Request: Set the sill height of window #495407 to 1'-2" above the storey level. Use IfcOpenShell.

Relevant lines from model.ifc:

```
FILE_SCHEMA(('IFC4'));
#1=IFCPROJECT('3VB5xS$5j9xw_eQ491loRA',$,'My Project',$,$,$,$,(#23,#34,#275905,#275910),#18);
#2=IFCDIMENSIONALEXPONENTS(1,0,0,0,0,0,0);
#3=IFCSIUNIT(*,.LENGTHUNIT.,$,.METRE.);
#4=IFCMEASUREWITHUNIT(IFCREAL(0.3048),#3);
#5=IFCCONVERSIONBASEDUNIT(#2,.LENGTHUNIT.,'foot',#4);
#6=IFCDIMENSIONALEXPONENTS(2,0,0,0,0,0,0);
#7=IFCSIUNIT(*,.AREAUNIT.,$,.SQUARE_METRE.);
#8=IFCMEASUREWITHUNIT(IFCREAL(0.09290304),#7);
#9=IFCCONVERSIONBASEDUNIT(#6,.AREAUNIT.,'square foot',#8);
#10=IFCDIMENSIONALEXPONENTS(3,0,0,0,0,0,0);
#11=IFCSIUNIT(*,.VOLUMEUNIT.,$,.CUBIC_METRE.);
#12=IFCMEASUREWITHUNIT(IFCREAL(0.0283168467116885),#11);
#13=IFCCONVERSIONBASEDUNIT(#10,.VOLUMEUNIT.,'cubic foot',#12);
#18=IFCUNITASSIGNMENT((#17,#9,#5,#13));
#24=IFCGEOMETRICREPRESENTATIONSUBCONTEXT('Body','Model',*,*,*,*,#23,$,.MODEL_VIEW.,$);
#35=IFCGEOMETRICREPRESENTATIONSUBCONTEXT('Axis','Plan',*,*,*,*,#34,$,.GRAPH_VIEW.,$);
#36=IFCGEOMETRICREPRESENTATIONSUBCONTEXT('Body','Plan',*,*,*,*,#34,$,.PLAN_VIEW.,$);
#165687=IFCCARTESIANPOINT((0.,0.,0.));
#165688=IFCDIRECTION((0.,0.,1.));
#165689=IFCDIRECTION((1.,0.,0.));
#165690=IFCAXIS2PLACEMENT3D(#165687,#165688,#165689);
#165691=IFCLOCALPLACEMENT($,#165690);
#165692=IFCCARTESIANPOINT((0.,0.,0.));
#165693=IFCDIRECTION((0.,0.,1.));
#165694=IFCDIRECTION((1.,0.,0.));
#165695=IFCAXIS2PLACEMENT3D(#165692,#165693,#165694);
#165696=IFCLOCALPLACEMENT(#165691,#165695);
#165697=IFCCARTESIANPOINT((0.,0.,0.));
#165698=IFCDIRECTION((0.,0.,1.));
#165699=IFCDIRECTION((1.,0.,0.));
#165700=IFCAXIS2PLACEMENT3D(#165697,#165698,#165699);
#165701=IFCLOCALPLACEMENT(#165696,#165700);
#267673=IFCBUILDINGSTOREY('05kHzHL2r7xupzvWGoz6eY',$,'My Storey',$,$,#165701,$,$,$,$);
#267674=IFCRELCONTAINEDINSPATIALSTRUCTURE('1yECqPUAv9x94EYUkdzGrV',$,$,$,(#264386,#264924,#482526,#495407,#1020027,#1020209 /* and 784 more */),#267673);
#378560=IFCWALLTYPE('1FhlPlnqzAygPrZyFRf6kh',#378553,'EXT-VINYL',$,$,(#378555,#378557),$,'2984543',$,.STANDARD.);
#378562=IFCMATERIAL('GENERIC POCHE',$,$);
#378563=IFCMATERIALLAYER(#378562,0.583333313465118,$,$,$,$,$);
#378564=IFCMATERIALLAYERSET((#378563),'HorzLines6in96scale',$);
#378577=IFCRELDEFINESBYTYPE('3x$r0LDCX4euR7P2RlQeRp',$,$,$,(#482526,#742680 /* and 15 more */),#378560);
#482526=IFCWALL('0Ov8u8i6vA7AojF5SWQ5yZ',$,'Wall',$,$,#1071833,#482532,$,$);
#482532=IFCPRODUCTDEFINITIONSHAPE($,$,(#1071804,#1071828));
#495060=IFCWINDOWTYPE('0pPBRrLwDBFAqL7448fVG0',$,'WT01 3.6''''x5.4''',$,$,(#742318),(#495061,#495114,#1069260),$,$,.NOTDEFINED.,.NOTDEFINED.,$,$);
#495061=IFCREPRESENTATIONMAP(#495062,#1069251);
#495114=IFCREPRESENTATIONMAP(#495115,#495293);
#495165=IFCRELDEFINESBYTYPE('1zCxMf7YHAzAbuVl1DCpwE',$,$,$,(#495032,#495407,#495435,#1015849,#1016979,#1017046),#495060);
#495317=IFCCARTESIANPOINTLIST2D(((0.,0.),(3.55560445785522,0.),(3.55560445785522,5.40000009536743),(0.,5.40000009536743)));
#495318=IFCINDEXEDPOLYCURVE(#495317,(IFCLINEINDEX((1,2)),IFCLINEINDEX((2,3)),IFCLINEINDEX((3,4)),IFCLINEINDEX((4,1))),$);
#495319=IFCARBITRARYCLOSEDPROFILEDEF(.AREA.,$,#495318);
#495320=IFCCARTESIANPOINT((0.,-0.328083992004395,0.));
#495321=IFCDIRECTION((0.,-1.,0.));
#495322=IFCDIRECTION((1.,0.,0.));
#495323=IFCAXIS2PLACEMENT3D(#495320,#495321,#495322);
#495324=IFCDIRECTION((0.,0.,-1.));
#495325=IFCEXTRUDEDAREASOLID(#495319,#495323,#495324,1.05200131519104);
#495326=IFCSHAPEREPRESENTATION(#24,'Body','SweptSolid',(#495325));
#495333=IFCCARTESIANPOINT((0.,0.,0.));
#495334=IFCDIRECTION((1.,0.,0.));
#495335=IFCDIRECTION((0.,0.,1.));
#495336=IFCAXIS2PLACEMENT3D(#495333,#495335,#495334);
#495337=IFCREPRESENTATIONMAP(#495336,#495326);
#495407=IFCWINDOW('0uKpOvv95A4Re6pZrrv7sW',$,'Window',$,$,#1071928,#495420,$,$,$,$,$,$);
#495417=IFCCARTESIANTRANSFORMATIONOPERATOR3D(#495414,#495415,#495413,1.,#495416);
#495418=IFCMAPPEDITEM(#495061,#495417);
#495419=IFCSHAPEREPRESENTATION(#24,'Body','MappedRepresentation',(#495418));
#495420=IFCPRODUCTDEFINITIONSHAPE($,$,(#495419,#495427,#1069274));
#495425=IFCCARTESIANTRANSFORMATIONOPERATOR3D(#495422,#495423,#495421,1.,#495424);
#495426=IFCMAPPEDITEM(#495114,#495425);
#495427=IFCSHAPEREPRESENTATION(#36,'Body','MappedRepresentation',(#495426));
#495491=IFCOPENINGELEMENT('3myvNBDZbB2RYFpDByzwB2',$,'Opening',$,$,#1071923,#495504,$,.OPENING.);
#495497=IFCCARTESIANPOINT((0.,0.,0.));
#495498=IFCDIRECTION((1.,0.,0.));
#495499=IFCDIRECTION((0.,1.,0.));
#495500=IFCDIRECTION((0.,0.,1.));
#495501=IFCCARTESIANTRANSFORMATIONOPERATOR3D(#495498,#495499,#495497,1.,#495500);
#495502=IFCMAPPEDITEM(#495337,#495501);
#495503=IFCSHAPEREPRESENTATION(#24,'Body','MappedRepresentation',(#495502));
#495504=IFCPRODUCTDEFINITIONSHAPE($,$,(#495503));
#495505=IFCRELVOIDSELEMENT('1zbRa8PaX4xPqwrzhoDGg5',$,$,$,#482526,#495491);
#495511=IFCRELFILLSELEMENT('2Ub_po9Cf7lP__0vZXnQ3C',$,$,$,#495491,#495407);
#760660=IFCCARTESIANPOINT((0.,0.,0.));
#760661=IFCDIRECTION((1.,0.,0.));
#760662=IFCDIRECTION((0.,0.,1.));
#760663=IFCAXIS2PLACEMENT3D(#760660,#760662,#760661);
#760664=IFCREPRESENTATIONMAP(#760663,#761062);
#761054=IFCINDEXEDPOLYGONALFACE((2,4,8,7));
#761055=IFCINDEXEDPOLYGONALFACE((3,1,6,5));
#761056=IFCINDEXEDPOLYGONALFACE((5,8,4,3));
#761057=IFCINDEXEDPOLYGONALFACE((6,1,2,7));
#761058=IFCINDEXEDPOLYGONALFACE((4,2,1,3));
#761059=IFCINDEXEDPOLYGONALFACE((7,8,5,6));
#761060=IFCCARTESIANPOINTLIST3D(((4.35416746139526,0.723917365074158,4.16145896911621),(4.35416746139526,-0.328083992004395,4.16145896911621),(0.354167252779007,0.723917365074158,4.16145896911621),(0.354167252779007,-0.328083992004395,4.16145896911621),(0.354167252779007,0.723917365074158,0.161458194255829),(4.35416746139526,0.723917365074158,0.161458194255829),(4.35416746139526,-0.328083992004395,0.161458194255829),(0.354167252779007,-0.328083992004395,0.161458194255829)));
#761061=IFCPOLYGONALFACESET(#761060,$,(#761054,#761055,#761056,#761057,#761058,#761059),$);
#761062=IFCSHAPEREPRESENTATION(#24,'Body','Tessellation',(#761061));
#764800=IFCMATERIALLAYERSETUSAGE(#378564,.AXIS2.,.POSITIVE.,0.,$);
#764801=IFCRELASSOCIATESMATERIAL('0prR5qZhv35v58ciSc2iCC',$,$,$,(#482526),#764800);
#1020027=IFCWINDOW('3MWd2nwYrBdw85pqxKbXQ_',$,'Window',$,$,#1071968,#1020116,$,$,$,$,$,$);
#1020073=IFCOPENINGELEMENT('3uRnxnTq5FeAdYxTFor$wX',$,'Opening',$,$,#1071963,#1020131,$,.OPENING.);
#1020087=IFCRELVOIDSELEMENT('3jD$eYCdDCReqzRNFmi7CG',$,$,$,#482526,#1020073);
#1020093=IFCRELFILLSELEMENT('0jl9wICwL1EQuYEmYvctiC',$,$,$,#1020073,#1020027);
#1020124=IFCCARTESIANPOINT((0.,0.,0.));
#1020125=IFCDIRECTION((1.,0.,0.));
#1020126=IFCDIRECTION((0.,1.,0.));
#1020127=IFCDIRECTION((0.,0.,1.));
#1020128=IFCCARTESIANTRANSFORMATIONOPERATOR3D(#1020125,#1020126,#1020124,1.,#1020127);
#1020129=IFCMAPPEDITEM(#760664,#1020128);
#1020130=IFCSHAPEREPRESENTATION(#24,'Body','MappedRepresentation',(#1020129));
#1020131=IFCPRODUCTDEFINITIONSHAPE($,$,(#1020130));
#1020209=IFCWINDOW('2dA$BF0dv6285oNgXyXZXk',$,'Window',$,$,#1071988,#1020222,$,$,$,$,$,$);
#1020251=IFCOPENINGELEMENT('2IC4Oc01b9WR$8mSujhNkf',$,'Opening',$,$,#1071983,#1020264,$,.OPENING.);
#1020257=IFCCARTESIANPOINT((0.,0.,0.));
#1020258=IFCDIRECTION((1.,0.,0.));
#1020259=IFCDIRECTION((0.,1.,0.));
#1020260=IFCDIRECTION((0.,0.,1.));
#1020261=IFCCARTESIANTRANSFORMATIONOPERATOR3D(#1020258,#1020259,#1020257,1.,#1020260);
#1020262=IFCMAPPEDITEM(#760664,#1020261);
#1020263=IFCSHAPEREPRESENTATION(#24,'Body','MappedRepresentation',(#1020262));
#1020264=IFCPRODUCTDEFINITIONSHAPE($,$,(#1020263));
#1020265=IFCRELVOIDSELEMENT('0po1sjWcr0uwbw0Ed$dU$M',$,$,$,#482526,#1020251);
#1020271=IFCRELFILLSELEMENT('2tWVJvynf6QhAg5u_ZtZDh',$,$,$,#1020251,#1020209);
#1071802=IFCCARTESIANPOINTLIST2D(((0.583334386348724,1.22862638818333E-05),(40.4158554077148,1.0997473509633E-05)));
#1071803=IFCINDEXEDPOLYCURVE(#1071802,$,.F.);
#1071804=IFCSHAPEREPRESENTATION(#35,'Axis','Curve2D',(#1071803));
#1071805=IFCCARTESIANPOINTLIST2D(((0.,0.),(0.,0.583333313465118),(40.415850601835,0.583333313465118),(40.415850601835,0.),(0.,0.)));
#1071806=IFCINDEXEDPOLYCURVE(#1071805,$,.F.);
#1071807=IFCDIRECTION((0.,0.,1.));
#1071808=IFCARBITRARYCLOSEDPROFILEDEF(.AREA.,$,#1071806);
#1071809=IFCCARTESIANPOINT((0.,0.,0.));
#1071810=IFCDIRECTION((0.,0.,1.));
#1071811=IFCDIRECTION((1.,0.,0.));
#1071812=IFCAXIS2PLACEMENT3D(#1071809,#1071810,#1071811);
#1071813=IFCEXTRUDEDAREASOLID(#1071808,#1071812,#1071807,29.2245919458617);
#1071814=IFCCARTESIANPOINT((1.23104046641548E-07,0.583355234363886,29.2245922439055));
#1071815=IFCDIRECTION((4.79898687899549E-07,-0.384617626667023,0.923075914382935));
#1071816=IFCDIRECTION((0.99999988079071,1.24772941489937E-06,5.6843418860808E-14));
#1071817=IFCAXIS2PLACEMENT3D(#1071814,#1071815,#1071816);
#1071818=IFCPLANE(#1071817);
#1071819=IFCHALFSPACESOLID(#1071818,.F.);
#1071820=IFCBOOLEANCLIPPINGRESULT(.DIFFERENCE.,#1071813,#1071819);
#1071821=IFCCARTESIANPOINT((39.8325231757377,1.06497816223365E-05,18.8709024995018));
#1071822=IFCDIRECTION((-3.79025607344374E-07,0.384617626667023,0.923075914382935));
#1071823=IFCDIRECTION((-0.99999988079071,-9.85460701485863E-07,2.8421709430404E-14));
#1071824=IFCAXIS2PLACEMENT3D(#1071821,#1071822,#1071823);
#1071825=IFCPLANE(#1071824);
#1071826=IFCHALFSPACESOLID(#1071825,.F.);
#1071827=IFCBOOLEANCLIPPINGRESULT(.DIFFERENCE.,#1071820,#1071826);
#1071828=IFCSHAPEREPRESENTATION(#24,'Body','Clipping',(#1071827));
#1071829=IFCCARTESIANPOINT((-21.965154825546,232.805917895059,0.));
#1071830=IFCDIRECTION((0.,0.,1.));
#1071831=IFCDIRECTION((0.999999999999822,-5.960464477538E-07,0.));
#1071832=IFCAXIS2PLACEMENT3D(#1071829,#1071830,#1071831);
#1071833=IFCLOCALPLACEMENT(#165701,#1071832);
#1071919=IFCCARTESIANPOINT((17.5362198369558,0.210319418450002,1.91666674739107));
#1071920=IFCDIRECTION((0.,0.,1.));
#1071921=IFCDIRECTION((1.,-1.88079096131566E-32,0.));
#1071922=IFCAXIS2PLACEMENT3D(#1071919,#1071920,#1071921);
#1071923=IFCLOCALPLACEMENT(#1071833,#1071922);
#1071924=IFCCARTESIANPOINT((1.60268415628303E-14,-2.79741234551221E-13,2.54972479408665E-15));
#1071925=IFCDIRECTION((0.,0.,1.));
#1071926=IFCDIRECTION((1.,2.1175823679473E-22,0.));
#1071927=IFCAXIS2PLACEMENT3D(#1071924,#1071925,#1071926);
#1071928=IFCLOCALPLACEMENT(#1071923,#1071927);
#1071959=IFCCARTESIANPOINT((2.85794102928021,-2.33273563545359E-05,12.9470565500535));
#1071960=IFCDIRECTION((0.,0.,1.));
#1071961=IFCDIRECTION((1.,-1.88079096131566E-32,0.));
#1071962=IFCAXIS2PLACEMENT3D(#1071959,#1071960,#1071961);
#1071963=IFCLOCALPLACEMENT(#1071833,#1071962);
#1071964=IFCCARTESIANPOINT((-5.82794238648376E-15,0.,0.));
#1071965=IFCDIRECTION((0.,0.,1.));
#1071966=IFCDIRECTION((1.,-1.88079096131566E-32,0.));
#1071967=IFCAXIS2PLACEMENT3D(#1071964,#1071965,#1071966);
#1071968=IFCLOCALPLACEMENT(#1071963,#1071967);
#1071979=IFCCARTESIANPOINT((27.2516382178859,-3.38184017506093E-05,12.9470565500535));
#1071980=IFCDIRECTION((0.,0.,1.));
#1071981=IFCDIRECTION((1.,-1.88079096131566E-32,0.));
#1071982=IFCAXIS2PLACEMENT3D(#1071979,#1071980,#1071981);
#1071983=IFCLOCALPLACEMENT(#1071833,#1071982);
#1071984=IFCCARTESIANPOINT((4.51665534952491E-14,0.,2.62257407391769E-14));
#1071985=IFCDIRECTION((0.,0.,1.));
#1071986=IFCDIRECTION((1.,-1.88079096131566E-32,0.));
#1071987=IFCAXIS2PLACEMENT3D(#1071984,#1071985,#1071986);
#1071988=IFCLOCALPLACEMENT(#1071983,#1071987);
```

```python
import numpy as np
import ifcopenshell
import ifcopenshell.api.geometry
import ifcopenshell.geom
import ifcopenshell.util.element
import ifcopenshell.util.placement
import ifcopenshell.util.shape
import ifcopenshell.util.unit

model = ifcopenshell.open("model.ifc")
unit_scale = ifcopenshell.util.unit.calculate_unit_scale(model)

window = model.by_guid("0uKpOvv95A4Re6pZrrv7sW")
opening = window.FillsVoids[0].RelatingOpeningElement
storey = ifcopenshell.util.element.get_container(window, ifc_class="IfcBuildingStorey")
level = ifcopenshell.util.placement.get_local_placement(storey.ObjectPlacement)[2, 3]

# The opening's origin need not be at the sill, so measure its lowest point.
shape = ifcopenshell.geom.create_shape(ifcopenshell.geom.settings(), opening)
bottom = ifcopenshell.util.shape.get_shape_bottom_elevation(shape, shape.geometry) / unit_scale
dz = level + 14 * 0.0254 / unit_scale - bottom

shift = np.array([0.0, 0.0, dz])
# The window is placed relative to its opening, so it follows when the opening moves.
matrix = ifcopenshell.util.placement.get_local_placement(opening.ObjectPlacement)
matrix[:3, 3] += shift
ifcopenshell.api.geometry.edit_object_placement(
    model, product=opening, matrix=matrix, is_si=False, should_transform_children=True
)

print(f"moved by {dz * unit_scale:+.3f} m")

model.write("model_v2.ifc")
```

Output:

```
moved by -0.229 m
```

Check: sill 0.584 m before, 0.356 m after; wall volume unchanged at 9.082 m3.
